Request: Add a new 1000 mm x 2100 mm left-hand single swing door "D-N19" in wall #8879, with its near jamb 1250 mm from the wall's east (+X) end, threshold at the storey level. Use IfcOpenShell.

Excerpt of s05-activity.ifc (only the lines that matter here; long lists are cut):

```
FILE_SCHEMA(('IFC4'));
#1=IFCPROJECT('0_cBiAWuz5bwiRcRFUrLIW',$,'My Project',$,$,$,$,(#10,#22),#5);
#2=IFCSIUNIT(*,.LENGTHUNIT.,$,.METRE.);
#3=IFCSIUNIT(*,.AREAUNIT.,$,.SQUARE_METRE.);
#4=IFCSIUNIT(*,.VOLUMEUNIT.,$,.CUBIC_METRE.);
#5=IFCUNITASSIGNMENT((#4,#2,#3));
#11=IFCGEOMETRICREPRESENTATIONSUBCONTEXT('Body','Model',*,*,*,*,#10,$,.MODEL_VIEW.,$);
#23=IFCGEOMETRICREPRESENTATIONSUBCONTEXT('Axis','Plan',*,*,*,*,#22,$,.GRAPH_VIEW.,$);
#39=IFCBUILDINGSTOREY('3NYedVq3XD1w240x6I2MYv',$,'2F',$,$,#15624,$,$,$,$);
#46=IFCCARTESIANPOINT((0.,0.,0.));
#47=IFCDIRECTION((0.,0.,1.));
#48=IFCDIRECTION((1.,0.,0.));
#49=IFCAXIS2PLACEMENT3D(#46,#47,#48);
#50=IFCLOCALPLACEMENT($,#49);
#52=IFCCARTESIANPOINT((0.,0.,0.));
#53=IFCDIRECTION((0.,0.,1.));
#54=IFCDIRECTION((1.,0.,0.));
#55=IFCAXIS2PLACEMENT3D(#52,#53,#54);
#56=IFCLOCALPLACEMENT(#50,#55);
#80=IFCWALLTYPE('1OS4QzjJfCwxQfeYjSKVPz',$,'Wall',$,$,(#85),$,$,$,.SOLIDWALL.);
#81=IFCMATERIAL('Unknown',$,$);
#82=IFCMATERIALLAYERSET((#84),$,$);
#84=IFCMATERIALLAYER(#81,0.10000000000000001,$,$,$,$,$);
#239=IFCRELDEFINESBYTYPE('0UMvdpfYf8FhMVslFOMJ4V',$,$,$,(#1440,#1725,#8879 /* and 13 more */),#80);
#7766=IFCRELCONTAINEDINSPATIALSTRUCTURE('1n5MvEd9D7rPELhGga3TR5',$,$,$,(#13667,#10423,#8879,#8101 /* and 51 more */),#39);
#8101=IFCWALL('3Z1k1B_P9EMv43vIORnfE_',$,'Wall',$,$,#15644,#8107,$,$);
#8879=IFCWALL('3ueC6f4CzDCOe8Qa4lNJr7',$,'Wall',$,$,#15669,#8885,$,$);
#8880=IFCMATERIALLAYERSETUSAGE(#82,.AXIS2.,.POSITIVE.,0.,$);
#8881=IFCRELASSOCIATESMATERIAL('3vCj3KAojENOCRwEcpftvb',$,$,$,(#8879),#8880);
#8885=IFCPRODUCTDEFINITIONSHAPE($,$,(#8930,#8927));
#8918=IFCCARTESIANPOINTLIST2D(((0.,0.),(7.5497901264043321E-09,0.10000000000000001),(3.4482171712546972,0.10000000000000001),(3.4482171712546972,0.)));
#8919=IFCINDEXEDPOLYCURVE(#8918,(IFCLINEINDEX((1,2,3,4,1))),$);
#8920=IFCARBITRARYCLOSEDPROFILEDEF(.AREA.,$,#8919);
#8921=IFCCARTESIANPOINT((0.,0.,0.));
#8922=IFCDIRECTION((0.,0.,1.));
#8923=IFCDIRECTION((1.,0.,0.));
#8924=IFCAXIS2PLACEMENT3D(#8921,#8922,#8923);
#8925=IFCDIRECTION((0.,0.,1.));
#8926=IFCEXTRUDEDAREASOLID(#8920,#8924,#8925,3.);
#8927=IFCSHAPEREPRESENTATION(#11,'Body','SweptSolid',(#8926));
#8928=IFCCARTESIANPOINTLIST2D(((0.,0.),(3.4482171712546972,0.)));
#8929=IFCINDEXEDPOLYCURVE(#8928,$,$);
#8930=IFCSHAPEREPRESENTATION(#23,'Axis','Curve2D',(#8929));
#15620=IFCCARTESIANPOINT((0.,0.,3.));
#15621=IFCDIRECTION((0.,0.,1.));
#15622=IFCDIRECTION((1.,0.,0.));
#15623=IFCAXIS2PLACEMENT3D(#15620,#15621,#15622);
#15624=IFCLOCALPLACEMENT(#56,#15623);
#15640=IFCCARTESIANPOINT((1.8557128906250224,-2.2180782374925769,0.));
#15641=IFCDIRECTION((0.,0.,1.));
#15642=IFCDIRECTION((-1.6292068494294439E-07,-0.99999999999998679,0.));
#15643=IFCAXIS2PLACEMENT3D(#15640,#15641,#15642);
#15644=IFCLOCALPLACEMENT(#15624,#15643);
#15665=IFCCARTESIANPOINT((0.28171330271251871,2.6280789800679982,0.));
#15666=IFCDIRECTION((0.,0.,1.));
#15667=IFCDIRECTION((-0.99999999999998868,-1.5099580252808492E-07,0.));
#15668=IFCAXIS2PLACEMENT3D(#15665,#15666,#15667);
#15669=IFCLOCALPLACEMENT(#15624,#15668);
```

```python
import numpy as np
import ifcopenshell
import ifcopenshell.api.feature
import ifcopenshell.api.geometry
import ifcopenshell.api.root
import ifcopenshell.api.spatial
import ifcopenshell.geom
import ifcopenshell.util.element
import ifcopenshell.util.placement
import ifcopenshell.util.representation
import ifcopenshell.util.shape
import ifcopenshell.util.unit

model = ifcopenshell.open("s05-activity.ifc")
unit_scale = ifcopenshell.util.unit.calculate_unit_scale(model)
settings = ifcopenshell.geom.settings()


def volume(element):
    """Net volume in cubic metres, openings subtracted."""
    shape = ifcopenshell.geom.create_shape(settings, element)
    return ifcopenshell.util.shape.get_volume(shape.geometry)


wall = model.by_guid("3ueC6f4CzDCOe8Qa4lNJr7")
storey = ifcopenshell.util.element.get_container(wall, ifc_class="IfcBuildingStorey")
context = ifcopenshell.util.representation.get_context(model, "Model", "Body", "MODEL_VIEW")
before = volume(wall)

width, height, from_end, sill = 1, 2.1, 1.25, 0.0  # metres

# The wall runs along its own X axis, and the end named is its -X end.
wall_shape = ifcopenshell.geom.create_shape(settings, wall)
x, y, z = ifcopenshell.util.shape.get_vertices(wall_shape.geometry).T
start = x.min() + from_end
face, thickness = float(y.min()), float(y.max() - y.min())
wall_matrix = ifcopenshell.util.placement.get_local_placement(wall.ObjectPlacement)
level = ifcopenshell.util.placement.get_local_placement(storey.ObjectPlacement)[2, 3]


def in_wall(x, y):
    """Placement at x, y metres in the wall's axes, at sill height."""
    matrix = wall_matrix.copy()
    matrix[:, 3] = wall_matrix @ np.array([x / unit_scale, y / unit_scale, 0.0, 1.0])
    matrix[2, 3] = level + sill / unit_scale
    return matrix


# Opening: a box that overshoots both wall faces by 50 mm.
opening = ifcopenshell.api.root.create_entity(model, ifc_class="IfcOpeningElement", predefined_type="OPENING")
box = ifcopenshell.api.geometry.add_wall_representation(
    model, context=context, length=width, height=height, thickness=thickness + 0.1
)
ifcopenshell.api.geometry.assign_representation(model, product=opening, representation=box)
ifcopenshell.api.geometry.edit_object_placement(model, product=opening, matrix=in_wall(start, face - 0.05), is_si=False)
ifcopenshell.api.feature.add_feature(model, feature=opening, element=wall)

door = ifcopenshell.api.root.create_entity(model, ifc_class="IfcDoor", name="D-N19", predefined_type="DOOR")
door.OverallWidth, door.OverallHeight = width / unit_scale, height / unit_scale
door.OperationType = "SINGLE_SWING_LEFT"
body = ifcopenshell.api.geometry.add_door_representation(
    model,
    context=context,
    overall_width=door.OverallWidth,
    overall_height=door.OverallHeight,
    operation_type="SINGLE_SWING_LEFT",
    lining_properties={"LiningDepth": thickness / unit_scale, "ThresholdDepth": thickness / unit_scale},
)
ifcopenshell.api.geometry.assign_representation(model, product=door, representation=body)
ifcopenshell.api.spatial.assign_container(model, products=[door], relating_structure=storey)
ifcopenshell.api.feature.add_filling(model, opening=opening, element=door)

# The lining spans the wall, so the door starts at the wall face.
ifcopenshell.api.geometry.edit_object_placement(model, product=door, matrix=in_wall(start, face), is_si=False)

after = volume(wall)

print(f"wall volume {before:.3f} -> {after:.3f} m3")

model.write("s05-activity_edited.ifc")
```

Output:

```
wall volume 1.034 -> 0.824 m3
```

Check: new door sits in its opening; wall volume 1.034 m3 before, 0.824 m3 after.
